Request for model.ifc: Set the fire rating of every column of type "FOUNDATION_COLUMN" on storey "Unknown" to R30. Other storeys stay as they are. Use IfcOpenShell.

First a look at what the model holds.

```python
import ifcopenshell
import ifcopenshell.util.element

model = ifcopenshell.open("model.ifc")
print(model.schema)
storey = next(s for s in model.by_type("IfcBuildingStorey") if s.Name == "Unknown")
columns = [e for e in ifcopenshell.util.element.get_decomposition(storey) if e.is_a("IfcColumn")]
seen = {}
for e in columns:
    element_type = ifcopenshell.util.element.get_type(e)
    key = (element_type.Name if element_type != e and element_type else None, ifcopenshell.util.element.get_pset(e, "Pset_ColumnCommon", "FireRating"))
    seen[key] = seen.get(key, 0) + 1
for (name, value), count in sorted(seen.items(), key=str):
    print(count, "x", name, "|", value)
```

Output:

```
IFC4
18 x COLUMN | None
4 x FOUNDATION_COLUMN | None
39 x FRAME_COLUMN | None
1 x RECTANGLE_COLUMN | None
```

```python
import ifcopenshell
import ifcopenshell.api.pset
import ifcopenshell.util.element

model = ifcopenshell.open("model.ifc")

storey = next(s for s in model.by_type("IfcBuildingStorey") if s.Name == "Unknown")
columns = [e for e in ifcopenshell.util.element.get_decomposition(storey) if e.is_a("IfcColumn")]

count = 0
for e in columns:
    element_type = ifcopenshell.util.element.get_type(e)
    if element_type in (None, e) or element_type.Name != "FOUNDATION_COLUMN":
        continue
    found = ifcopenshell.util.element.get_pset(e, "Pset_ColumnCommon", should_inherit=False)
    if found:
        pset = model.by_id(found["id"])
        if len(ifcopenshell.util.element.get_elements_by_pset(pset)) > 1:
            pset = ifcopenshell.api.pset.unshare_pset(model, products=[e], pset=pset)[0]
    else:
        pset = ifcopenshell.api.pset.add_pset(model, product=e, name="Pset_ColumnCommon")
    ifcopenshell.api.pset.edit_pset(model, pset=pset, properties={"FireRating": "R30"})
    count += 1

print(count, "columns updated")

model.write("model_updated.ifc")
```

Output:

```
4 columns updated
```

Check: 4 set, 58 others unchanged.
